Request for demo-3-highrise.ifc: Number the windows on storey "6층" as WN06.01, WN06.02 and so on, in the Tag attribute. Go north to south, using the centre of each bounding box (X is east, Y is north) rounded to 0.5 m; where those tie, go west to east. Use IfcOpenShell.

First a look at what the model holds.

```python
import ifcopenshell
import ifcopenshell.util.element
import ifcopenshell.util.placement

model = ifcopenshell.open("demo-3-highrise.ifc")
print(model.schema)
storey = next(s for s in model.by_type("IfcBuildingStorey") if s.Name == "6층")
windows = [e for e in ifcopenshell.util.element.get_decomposition(storey) if e.is_a("IfcWindow")]
for e in sorted(windows, key=lambda e: e.id()):
    origin = ifcopenshell.util.placement.get_local_placement(e.ObjectPlacement)[:3, 3]
    print(e.id(), e.Tag, e.Name, origin.round(2) + 0.0, sep=" | ")
```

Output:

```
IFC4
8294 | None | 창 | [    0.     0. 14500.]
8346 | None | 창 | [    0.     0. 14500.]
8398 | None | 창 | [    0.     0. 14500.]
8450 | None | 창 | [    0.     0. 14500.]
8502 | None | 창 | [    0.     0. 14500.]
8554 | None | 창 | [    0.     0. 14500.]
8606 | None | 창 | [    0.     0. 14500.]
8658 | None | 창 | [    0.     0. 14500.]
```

```python
import ifcopenshell
import ifcopenshell.geom
import ifcopenshell.util.element
import ifcopenshell.util.shape

model = ifcopenshell.open("demo-3-highrise.ifc")
settings = ifcopenshell.geom.settings()
settings.set("use-world-coords", True)


def centre(element):
    shape = ifcopenshell.geom.create_shape(settings, element)
    return ifcopenshell.util.shape.get_bbox_centroid(shape.geometry)


storey = next(s for s in model.by_type("IfcBuildingStorey") if s.Name == "6층")
windows = [e for e in ifcopenshell.util.element.get_decomposition(storey) if e.is_a("IfcWindow")]

# Insertion points can sit at a corner or the storey origin, so sort by the geometry (in metres).
centres = {e: centre(e) for e in windows}
windows.sort(key=lambda e: (-round(centres[e][1] / 0.5), centres[e][0]))

for i, e in enumerate(windows, start=1):
    number = f"WN06.{i:02d}"
    e.Tag = number
    print(e.id(), number)

model.write("demo-3-highrise_edited.ifc")
```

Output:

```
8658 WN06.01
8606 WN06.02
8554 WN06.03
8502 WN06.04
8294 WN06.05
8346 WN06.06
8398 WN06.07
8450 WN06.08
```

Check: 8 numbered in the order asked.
